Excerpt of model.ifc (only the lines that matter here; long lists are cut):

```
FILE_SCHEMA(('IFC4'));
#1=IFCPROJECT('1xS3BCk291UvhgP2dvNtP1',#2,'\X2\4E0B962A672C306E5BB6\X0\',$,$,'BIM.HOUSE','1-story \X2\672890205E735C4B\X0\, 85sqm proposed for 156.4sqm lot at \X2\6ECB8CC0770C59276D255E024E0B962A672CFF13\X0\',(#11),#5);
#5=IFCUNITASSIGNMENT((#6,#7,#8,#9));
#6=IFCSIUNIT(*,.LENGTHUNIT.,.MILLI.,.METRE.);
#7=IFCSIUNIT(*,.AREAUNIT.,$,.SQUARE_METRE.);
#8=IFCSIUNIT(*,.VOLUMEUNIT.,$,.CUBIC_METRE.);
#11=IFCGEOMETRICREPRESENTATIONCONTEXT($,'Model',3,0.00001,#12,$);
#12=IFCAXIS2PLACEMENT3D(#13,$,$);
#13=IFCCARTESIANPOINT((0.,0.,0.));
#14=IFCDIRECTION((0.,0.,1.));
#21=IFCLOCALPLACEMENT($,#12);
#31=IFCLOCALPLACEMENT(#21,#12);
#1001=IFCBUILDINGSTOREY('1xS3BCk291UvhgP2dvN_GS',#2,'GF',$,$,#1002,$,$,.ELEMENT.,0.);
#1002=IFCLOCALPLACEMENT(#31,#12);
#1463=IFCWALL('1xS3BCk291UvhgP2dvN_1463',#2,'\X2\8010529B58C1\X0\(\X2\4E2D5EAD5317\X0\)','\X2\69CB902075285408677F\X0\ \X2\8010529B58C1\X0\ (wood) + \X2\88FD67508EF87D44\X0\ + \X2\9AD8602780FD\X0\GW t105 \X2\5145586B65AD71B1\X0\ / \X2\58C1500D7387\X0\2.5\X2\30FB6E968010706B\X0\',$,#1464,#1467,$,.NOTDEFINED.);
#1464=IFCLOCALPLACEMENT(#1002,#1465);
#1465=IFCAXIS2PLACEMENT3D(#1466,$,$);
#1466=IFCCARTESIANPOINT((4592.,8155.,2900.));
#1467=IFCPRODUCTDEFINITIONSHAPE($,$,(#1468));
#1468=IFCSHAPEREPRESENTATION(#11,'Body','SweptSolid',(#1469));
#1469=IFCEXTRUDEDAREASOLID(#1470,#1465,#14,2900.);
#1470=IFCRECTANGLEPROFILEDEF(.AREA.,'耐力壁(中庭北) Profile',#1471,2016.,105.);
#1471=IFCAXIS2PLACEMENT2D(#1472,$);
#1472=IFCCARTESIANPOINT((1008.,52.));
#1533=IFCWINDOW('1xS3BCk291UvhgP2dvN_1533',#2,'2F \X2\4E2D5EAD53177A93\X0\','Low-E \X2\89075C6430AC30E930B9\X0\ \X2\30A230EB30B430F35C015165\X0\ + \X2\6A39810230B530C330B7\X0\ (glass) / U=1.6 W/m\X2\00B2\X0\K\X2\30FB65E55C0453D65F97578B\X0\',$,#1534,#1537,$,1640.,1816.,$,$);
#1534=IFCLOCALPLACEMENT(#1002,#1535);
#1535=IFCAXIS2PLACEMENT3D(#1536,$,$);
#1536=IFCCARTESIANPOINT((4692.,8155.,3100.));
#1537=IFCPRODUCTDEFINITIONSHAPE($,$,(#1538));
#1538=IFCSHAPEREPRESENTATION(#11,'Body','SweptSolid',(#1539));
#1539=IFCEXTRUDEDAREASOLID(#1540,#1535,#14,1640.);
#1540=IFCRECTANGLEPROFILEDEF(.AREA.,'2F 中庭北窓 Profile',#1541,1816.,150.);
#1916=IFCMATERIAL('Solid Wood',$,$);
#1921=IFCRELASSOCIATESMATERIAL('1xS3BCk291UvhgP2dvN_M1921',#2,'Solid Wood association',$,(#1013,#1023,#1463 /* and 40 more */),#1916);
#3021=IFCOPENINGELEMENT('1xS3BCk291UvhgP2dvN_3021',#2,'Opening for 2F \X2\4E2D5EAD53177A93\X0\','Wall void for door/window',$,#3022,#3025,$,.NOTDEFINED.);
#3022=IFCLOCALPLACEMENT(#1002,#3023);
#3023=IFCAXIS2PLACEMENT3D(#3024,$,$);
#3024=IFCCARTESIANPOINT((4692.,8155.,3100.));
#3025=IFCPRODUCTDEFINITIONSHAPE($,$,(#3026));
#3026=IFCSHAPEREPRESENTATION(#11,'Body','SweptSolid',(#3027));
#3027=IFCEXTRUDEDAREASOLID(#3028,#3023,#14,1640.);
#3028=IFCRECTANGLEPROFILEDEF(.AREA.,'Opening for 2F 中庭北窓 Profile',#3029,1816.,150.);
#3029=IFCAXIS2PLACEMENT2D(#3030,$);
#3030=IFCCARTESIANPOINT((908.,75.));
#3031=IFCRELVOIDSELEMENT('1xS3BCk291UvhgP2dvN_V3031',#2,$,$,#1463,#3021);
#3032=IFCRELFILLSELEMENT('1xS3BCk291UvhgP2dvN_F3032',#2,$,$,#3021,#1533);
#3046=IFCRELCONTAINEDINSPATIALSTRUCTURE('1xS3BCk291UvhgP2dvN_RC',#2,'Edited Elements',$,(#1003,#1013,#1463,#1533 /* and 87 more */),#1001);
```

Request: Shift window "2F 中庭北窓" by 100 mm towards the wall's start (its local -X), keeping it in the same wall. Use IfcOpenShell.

```python
import ifcopenshell
import ifcopenshell.api.geometry
import ifcopenshell.util.placement
import ifcopenshell.util.unit

model = ifcopenshell.open("model.ifc")
unit_scale = ifcopenshell.util.unit.calculate_unit_scale(model)

window = model.by_id(1533)
opening = window.FillsVoids[0].RelatingOpeningElement
wall = opening.VoidsElements[0].RelatingBuildingElement

wall_matrix = ifcopenshell.util.placement.get_local_placement(wall.ObjectPlacement)
shift = wall_matrix[:3, 0] * -0.1 / unit_scale
before = ifcopenshell.util.placement.get_local_placement(window.ObjectPlacement)[:3, 3].copy()

# The window is not placed relative to its opening, so move both.
for product in (opening, window):
    matrix = ifcopenshell.util.placement.get_local_placement(product.ObjectPlacement)
    matrix[:3, 3] += shift
    ifcopenshell.api.geometry.edit_object_placement(model, product=product, matrix=matrix, is_si=False)

after = ifcopenshell.util.placement.get_local_placement(window.ObjectPlacement)[:3, 3]
print("window moved by", (after - before).round(3) + 0.0)

model.write("model_v2.ifc")
```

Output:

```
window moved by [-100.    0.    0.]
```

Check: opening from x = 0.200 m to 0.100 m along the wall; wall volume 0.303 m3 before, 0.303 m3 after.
